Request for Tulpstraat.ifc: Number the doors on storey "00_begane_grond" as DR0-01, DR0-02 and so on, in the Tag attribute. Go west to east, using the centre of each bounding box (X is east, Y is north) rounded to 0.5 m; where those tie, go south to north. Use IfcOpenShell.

First a look at what the model holds.

```python
import ifcopenshell
import ifcopenshell.util.element
import ifcopenshell.util.placement

model = ifcopenshell.open("Tulpstraat.ifc")
print(model.schema)
storey = next(s for s in model.by_type("IfcBuildingStorey") if s.Name == "00_begane_grond")
doors = [e for e in ifcopenshell.util.element.get_decomposition(storey) if e.is_a("IfcDoor")]
for e in sorted(doors, key=lambda e: e.id()):
    origin = ifcopenshell.util.placement.get_local_placement(e.ObjectPlacement)[:3, 3]
    print(e.id(), e.Tag, e.Name, origin.round(2) + 0.0, sep=" | ")
```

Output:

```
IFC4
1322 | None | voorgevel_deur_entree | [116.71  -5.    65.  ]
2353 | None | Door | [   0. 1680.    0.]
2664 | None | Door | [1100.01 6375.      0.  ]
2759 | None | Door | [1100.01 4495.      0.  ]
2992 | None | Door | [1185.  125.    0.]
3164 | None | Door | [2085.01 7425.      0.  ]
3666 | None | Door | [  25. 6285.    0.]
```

```python
import ifcopenshell
import ifcopenshell.geom
import ifcopenshell.util.element
import ifcopenshell.util.shape

model = ifcopenshell.open("Tulpstraat.ifc")
settings = ifcopenshell.geom.settings()
settings.set("use-world-coords", True)


def centre(element):
    shape = ifcopenshell.geom.create_shape(settings, element)
    return ifcopenshell.util.shape.get_bbox_centroid(shape.geometry)


storey = next(s for s in model.by_type("IfcBuildingStorey") if s.Name == "00_begane_grond")
doors = [e for e in ifcopenshell.util.element.get_decomposition(storey) if e.is_a("IfcDoor")]

# Insertion points can sit at a corner or the storey origin, so sort by the geometry (in metres).
centres = {e: centre(e) for e in doors}
doors.sort(key=lambda e: (round(centres[e][0] / 0.5), centres[e][1]))

for i, e in enumerate(doors, start=1):
    number = f"DR0-{i:02d}"
    e.Tag = number
    print(e.id(), number)

model.write("Tulpstraat-out.ifc")
```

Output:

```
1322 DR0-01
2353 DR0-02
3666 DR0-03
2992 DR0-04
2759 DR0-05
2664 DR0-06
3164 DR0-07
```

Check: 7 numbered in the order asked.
